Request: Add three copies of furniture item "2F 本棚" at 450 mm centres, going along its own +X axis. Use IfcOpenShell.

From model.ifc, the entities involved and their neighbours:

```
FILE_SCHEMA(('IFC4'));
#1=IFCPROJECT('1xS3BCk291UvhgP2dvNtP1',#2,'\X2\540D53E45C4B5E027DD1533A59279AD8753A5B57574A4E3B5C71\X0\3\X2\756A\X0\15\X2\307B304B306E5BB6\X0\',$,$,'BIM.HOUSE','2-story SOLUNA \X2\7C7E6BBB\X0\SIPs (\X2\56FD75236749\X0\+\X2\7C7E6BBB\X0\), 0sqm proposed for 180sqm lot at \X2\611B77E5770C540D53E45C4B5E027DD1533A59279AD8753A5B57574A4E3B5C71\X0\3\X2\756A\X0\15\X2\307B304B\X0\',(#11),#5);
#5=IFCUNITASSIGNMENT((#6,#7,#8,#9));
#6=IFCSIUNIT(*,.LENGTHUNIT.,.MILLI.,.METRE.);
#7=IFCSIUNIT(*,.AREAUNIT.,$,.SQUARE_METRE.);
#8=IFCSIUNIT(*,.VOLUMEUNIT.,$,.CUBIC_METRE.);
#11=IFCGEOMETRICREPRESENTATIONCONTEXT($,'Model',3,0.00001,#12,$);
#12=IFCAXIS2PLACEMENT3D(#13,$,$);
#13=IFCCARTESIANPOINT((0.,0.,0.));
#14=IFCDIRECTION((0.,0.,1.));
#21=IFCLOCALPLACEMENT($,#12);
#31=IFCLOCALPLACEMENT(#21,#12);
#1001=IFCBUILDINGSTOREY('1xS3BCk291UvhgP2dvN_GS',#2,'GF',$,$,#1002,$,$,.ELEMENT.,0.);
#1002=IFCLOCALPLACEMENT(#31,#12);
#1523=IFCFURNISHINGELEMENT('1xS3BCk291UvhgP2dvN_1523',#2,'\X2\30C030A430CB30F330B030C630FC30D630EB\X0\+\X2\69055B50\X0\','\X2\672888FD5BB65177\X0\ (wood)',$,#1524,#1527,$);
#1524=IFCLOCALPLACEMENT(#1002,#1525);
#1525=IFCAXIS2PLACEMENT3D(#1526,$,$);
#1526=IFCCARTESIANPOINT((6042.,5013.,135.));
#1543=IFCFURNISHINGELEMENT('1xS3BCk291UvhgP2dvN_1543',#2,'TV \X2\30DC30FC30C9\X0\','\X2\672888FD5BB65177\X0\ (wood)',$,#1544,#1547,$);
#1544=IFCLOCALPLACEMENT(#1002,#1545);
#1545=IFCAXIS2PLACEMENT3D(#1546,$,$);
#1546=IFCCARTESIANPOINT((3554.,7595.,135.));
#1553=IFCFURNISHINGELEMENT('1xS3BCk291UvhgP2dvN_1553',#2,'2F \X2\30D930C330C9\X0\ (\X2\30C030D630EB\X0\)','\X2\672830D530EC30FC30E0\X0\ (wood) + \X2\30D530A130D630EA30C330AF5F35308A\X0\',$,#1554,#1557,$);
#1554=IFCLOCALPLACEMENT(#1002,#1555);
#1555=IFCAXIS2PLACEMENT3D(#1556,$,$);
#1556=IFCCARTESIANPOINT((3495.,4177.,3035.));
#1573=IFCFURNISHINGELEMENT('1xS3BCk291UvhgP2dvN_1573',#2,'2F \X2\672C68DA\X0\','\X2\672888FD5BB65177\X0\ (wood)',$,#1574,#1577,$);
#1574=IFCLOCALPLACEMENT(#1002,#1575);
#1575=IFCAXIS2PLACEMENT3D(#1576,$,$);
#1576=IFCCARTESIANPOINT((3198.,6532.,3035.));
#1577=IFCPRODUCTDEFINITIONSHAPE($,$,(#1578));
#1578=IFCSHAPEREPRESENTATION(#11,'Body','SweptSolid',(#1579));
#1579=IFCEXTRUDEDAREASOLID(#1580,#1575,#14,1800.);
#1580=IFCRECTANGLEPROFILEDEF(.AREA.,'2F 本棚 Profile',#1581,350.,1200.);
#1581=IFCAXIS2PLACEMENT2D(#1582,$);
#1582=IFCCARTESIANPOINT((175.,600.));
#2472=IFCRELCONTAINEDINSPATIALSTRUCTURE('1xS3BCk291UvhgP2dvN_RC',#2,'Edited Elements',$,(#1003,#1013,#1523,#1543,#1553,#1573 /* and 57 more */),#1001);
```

```python
import ifcopenshell
import ifcopenshell.api.geometry
import ifcopenshell.api.root
import ifcopenshell.util.element
import ifcopenshell.util.placement

model = ifcopenshell.open("model.ifc")


def reuse_history(source, copy):
    """copy_class also copies each property set's owner history, people and application; keep the originals."""
    for rel in copy.IsDefinedBy:
        if rel.is_a("IfcRelDefinesByProperties") and (history := rel.RelatingPropertyDefinition.OwnerHistory):
            rel.RelatingPropertyDefinition.OwnerHistory = source.OwnerHistory
            ifcopenshell.util.element.remove_deep2(model, history)


source = model.by_guid("1xS3BCk291UvhgP2dvN_1573")
base = ifcopenshell.util.placement.get_local_placement(source.ObjectPlacement)
step = base[:3, 0] * 450.0

for i in range(1, 4):
    copy = ifcopenshell.api.root.copy_class(model, product=source)
    copy.Representation = ifcopenshell.util.element.copy_deep(
        model, source.Representation, exclude=["IfcGeometricRepresentationContext", "IfcRepresentationMap"]
    )
    reuse_history(source, copy)
    matrix = base.copy()
    matrix[:3, 3] += i * step
    print("added at", matrix[:3, 3].round(3) + 0.0)
    ifcopenshell.api.geometry.edit_object_placement(model, product=copy, matrix=matrix, is_si=False)

model.write("model_rev.ifc")
```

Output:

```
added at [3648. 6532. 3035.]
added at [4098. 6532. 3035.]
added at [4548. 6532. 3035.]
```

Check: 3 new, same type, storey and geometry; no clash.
